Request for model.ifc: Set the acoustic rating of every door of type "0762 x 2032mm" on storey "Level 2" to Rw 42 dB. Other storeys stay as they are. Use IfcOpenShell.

First a look at what the model holds.

```python
import ifcopenshell
import ifcopenshell.util.element

model = ifcopenshell.open("model.ifc")
print(model.schema)
storey = next(s for s in model.by_type("IfcBuildingStorey") if s.Name == "Level 2")
doors = [e for e in ifcopenshell.util.element.get_decomposition(storey) if e.is_a("IfcDoor")]
seen = {}
for e in doors:
    element_type = ifcopenshell.util.element.get_type(e)
    key = (element_type.Name if element_type != e and element_type else None, ifcopenshell.util.element.get_pset(e, "Pset_DoorCommon", "AcousticRating"))
    seen[key] = seen.get(key, 0) + 1
for (name, value), count in sorted(seen.items(), key=str):
    print(count, "x", name, "|", value)
```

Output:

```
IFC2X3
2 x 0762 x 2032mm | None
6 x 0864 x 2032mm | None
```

```python
import ifcopenshell
import ifcopenshell.api.pset
import ifcopenshell.util.element

model = ifcopenshell.open("model.ifc")

storey = next(s for s in model.by_type("IfcBuildingStorey") if s.Name == "Level 2")
doors = [e for e in ifcopenshell.util.element.get_decomposition(storey) if e.is_a("IfcDoor")]

count = 0
for e in doors:
    element_type = ifcopenshell.util.element.get_type(e)
    if element_type in (None, e) or element_type.Name != "0762 x 2032mm":
        continue
    # add_pset returns the element's existing set when there is one.
    pset = ifcopenshell.api.pset.add_pset(model, product=e, name="Pset_DoorCommon")
    ifcopenshell.api.pset.edit_pset(model, pset=pset, properties={"AcousticRating": "Rw 42 dB"})
    count += 1

print(count, "doors updated")

model.write("model_v2.ifc")
```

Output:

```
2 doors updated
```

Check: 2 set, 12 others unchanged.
